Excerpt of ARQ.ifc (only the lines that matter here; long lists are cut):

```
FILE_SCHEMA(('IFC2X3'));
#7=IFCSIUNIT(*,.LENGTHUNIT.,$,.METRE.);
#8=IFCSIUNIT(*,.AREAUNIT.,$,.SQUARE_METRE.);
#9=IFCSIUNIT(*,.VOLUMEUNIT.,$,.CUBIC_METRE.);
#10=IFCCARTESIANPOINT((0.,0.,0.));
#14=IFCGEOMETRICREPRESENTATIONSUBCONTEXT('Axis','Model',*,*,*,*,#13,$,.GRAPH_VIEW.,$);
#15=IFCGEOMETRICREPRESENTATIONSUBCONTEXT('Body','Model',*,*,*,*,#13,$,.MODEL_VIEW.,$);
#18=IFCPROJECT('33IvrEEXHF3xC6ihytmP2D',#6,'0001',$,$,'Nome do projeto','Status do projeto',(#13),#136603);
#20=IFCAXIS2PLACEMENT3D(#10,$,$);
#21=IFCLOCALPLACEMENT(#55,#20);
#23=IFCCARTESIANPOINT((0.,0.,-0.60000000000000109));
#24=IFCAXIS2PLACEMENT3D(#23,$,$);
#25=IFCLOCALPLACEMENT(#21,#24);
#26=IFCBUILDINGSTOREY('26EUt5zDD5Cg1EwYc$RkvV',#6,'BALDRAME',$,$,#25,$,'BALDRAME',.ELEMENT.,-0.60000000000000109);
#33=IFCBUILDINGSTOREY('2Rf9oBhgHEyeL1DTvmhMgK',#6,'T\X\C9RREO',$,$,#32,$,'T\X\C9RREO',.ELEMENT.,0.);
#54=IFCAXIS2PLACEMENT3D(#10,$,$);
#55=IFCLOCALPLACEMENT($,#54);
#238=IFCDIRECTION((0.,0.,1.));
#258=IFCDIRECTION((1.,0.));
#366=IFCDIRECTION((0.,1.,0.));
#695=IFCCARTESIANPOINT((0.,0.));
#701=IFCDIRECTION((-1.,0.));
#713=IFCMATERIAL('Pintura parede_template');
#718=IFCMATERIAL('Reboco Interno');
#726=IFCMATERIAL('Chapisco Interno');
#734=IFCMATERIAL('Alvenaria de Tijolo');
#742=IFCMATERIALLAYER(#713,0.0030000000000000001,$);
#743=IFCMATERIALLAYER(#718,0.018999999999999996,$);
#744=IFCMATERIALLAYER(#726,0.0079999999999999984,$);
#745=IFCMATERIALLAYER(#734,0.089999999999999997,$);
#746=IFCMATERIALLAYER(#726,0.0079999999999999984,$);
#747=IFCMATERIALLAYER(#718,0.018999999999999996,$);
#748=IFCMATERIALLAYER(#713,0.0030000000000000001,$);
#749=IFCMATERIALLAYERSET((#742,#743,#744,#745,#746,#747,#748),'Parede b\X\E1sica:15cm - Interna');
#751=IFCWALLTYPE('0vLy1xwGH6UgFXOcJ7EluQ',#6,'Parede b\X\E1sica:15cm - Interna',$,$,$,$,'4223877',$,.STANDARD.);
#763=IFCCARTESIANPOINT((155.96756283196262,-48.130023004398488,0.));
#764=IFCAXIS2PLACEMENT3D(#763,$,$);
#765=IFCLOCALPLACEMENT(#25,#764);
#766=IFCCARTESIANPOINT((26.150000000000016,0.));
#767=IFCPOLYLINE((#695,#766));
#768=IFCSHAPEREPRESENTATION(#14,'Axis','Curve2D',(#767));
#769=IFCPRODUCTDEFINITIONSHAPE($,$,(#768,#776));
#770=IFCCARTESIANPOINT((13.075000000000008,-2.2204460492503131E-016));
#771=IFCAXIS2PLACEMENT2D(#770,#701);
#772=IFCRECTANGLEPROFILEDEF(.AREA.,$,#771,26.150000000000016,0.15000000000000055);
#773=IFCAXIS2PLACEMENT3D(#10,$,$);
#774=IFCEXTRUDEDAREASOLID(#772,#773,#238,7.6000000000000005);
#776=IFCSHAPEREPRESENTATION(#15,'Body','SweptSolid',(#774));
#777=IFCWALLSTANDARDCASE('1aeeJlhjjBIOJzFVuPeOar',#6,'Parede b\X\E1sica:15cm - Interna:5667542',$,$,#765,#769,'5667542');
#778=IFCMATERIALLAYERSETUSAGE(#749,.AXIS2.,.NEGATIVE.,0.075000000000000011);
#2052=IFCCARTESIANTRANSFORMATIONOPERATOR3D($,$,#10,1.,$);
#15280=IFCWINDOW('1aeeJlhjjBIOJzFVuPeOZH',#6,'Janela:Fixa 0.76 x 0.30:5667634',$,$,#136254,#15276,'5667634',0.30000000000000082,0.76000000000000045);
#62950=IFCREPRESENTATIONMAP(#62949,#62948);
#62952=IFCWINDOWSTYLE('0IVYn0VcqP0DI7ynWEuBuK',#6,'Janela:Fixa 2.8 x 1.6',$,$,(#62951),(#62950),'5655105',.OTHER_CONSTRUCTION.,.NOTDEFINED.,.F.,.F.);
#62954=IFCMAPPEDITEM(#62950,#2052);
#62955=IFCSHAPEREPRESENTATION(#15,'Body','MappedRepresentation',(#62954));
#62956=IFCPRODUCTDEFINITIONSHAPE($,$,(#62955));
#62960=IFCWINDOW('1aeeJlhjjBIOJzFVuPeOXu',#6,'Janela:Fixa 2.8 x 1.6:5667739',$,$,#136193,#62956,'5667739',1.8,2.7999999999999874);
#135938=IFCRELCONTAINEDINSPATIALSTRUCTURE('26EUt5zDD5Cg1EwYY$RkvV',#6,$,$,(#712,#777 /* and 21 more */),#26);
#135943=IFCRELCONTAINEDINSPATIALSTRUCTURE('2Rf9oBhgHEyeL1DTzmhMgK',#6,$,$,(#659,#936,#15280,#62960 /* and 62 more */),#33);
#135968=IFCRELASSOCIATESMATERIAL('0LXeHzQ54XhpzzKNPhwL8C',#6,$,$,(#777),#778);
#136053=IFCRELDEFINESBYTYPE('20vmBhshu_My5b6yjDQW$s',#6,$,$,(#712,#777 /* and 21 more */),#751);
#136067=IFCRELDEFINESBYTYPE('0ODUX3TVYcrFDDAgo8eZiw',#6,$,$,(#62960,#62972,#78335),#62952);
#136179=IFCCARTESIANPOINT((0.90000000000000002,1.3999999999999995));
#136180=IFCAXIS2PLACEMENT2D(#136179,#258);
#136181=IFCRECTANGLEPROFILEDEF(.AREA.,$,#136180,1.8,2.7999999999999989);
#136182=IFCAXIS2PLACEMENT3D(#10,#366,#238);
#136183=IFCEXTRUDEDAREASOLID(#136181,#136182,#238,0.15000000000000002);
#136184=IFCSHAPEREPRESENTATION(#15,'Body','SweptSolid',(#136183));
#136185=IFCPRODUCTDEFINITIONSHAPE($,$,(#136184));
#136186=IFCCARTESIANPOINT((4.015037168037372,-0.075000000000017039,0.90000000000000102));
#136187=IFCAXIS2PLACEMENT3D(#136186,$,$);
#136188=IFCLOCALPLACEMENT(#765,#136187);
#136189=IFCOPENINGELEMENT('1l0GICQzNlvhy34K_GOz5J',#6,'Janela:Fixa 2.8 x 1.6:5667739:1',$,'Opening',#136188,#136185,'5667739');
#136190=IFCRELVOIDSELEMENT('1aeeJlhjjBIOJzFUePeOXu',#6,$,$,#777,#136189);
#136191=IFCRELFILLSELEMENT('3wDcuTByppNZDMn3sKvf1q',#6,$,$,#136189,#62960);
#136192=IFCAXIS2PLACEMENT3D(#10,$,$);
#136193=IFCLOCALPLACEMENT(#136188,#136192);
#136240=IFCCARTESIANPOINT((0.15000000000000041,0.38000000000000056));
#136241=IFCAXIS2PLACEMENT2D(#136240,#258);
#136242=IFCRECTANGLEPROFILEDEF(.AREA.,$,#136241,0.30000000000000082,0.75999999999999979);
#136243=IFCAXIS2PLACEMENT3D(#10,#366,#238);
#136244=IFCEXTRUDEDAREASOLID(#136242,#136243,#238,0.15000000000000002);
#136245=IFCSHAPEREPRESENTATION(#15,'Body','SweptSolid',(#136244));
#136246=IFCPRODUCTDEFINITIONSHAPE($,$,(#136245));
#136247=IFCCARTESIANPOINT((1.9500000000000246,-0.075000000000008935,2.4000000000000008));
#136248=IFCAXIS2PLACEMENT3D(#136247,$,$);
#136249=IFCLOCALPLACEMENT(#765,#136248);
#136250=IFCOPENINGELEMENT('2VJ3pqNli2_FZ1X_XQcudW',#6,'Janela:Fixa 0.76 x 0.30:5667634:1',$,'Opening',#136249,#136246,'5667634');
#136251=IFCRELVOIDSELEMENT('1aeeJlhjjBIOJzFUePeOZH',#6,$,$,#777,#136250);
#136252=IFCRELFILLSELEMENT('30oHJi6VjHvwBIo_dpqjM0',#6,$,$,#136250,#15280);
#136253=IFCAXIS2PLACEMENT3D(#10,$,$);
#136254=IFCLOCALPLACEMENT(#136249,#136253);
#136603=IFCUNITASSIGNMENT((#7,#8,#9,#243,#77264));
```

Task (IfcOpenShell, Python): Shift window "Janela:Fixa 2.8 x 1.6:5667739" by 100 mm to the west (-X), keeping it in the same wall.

```python
import ifcopenshell
import ifcopenshell.api.geometry
import ifcopenshell.util.placement

model = ifcopenshell.open("ARQ.ifc")

window = model.by_id(62960)
opening = window.FillsVoids[0].RelatingOpeningElement
wall = opening.VoidsElements[0].RelatingBuildingElement

wall_matrix = ifcopenshell.util.placement.get_local_placement(wall.ObjectPlacement)
shift = wall_matrix[:3, 0] * -0.1
before = ifcopenshell.util.placement.get_local_placement(window.ObjectPlacement)[:3, 3].copy()

# The window is placed relative to its opening, so it follows when the opening moves.
matrix = ifcopenshell.util.placement.get_local_placement(opening.ObjectPlacement)
matrix[:3, 3] += shift
ifcopenshell.api.geometry.edit_object_placement(
    model, product=opening, matrix=matrix, is_si=False, should_transform_children=True
)

after = ifcopenshell.util.placement.get_local_placement(window.ObjectPlacement)[:3, 3]
print("window moved by", (after - before).round(3) + 0.0)

model.write("ARQ-out.ifc")
```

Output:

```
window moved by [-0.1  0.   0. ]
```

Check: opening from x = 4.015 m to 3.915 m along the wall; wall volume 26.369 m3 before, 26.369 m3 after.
